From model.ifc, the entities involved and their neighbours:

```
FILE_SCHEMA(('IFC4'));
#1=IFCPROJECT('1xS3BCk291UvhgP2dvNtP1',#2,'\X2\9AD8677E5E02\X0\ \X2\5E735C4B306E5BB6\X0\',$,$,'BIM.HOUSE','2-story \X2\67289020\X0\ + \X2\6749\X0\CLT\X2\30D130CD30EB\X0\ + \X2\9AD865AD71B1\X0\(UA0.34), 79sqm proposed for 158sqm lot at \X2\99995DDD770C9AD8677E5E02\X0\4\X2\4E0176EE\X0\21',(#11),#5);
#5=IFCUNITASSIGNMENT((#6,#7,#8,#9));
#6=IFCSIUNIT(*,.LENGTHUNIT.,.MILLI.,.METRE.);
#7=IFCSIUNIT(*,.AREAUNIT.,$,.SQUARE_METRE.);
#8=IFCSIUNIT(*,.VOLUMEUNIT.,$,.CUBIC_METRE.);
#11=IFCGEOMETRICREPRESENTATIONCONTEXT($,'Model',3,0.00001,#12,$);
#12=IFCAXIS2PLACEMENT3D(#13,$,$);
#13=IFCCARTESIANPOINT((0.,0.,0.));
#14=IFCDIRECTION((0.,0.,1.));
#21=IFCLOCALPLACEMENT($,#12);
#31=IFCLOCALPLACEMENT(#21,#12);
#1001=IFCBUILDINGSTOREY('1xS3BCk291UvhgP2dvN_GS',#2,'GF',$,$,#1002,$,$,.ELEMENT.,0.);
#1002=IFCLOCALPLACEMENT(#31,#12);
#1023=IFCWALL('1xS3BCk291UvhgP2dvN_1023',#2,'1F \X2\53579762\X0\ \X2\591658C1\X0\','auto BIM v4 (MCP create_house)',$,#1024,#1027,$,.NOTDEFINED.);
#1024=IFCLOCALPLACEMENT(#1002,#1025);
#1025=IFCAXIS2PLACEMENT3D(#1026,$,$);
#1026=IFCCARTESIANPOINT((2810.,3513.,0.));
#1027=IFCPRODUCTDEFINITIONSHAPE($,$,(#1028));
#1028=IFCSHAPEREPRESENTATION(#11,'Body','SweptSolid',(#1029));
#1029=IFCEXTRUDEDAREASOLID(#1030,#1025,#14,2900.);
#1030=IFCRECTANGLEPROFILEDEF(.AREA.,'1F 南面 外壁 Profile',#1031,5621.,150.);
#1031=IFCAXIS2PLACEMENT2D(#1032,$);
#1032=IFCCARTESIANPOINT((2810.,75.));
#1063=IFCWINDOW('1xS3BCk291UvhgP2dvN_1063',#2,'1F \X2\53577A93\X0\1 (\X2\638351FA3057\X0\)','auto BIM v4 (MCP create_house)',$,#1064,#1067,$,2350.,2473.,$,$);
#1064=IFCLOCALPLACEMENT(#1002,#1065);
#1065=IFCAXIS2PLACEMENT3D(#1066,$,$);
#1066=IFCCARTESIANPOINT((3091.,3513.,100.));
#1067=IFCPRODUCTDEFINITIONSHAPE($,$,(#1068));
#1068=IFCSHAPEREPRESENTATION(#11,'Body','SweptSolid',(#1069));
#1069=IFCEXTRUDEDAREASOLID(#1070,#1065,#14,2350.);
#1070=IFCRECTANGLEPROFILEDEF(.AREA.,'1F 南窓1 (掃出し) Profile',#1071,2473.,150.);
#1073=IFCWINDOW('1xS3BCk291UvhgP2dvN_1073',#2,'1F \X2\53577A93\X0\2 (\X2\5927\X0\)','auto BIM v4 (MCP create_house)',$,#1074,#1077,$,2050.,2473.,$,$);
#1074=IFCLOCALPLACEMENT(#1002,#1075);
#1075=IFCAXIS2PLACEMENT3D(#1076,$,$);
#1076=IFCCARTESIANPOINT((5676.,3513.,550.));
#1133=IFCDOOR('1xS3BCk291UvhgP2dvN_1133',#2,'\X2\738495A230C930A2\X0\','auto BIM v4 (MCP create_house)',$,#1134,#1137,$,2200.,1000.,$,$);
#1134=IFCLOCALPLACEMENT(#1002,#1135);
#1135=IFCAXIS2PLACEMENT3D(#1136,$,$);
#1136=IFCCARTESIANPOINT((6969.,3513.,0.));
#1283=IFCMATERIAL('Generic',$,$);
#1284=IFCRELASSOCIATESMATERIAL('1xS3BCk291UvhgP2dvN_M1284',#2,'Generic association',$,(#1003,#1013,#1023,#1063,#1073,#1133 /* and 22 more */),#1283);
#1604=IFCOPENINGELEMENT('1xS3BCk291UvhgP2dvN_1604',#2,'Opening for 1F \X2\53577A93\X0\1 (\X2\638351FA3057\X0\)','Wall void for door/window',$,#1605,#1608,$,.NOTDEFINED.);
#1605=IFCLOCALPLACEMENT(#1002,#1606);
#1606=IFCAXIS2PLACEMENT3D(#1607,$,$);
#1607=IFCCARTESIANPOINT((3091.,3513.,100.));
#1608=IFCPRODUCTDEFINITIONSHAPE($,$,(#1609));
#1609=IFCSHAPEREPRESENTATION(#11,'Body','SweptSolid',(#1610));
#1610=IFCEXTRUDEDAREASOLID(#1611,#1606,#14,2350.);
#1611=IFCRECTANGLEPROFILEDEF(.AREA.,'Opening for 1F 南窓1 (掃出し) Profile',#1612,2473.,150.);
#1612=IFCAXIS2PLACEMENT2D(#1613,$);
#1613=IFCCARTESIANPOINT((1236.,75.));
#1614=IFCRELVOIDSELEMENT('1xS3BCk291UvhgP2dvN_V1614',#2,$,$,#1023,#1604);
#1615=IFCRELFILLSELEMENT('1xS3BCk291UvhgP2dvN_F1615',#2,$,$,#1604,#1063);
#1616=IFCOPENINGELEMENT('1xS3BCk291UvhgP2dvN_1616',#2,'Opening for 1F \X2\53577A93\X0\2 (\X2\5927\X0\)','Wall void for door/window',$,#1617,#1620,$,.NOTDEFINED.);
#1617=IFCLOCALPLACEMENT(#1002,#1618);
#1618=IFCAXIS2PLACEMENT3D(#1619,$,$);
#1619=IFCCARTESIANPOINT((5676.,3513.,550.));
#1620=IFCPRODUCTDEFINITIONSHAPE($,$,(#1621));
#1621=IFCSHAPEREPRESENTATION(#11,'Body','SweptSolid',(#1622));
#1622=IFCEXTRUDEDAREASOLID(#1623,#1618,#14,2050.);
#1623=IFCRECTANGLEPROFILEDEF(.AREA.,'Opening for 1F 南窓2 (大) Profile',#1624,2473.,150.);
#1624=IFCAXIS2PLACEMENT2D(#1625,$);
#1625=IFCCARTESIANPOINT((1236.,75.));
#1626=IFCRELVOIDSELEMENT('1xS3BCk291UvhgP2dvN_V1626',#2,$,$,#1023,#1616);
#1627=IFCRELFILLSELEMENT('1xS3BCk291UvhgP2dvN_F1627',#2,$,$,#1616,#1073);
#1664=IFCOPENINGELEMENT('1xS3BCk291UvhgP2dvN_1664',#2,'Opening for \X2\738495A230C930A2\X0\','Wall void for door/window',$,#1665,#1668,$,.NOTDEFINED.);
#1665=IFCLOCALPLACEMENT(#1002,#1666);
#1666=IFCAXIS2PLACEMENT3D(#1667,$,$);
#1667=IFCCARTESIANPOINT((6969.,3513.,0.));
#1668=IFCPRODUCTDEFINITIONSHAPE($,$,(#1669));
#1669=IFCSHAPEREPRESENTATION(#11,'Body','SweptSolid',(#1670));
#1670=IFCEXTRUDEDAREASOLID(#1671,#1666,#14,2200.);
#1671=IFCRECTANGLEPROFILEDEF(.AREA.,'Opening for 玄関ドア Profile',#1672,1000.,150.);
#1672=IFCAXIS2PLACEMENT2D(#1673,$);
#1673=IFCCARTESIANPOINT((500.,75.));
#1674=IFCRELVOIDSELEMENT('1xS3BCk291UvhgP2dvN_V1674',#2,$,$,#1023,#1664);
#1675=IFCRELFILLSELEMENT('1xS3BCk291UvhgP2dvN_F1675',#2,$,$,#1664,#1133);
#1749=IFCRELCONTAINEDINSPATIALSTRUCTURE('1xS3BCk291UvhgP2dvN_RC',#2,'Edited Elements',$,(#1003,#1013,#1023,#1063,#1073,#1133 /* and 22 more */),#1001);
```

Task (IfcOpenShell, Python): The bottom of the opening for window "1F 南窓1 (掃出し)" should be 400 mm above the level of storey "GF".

```python
import numpy as np
import ifcopenshell
import ifcopenshell.api.geometry
import ifcopenshell.geom
import ifcopenshell.util.element
import ifcopenshell.util.placement
import ifcopenshell.util.shape
import ifcopenshell.util.unit

model = ifcopenshell.open("model.ifc")
unit_scale = ifcopenshell.util.unit.calculate_unit_scale(model)

window = model.by_id(1063)
opening = window.FillsVoids[0].RelatingOpeningElement
storey = ifcopenshell.util.element.get_container(window, ifc_class="IfcBuildingStorey")
level = ifcopenshell.util.placement.get_local_placement(storey.ObjectPlacement)[2, 3]

# The opening's origin need not be at the sill, so measure its lowest point.
shape = ifcopenshell.geom.create_shape(ifcopenshell.geom.settings(), opening)
bottom = ifcopenshell.util.shape.get_shape_bottom_elevation(shape, shape.geometry) / unit_scale
dz = level + 400.0 - bottom

shift = np.array([0.0, 0.0, dz])
# The window is not placed relative to its opening, so move both.
for product in (opening, window):
    matrix = ifcopenshell.util.placement.get_local_placement(product.ObjectPlacement)
    matrix[:3, 3] += shift
    ifcopenshell.api.geometry.edit_object_placement(model, product=product, matrix=matrix, is_si=False)

print(f"moved by {dz * unit_scale:+.3f} m")

model.write("model_updated.ifc")
```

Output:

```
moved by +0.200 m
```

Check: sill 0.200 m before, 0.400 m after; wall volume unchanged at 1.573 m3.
